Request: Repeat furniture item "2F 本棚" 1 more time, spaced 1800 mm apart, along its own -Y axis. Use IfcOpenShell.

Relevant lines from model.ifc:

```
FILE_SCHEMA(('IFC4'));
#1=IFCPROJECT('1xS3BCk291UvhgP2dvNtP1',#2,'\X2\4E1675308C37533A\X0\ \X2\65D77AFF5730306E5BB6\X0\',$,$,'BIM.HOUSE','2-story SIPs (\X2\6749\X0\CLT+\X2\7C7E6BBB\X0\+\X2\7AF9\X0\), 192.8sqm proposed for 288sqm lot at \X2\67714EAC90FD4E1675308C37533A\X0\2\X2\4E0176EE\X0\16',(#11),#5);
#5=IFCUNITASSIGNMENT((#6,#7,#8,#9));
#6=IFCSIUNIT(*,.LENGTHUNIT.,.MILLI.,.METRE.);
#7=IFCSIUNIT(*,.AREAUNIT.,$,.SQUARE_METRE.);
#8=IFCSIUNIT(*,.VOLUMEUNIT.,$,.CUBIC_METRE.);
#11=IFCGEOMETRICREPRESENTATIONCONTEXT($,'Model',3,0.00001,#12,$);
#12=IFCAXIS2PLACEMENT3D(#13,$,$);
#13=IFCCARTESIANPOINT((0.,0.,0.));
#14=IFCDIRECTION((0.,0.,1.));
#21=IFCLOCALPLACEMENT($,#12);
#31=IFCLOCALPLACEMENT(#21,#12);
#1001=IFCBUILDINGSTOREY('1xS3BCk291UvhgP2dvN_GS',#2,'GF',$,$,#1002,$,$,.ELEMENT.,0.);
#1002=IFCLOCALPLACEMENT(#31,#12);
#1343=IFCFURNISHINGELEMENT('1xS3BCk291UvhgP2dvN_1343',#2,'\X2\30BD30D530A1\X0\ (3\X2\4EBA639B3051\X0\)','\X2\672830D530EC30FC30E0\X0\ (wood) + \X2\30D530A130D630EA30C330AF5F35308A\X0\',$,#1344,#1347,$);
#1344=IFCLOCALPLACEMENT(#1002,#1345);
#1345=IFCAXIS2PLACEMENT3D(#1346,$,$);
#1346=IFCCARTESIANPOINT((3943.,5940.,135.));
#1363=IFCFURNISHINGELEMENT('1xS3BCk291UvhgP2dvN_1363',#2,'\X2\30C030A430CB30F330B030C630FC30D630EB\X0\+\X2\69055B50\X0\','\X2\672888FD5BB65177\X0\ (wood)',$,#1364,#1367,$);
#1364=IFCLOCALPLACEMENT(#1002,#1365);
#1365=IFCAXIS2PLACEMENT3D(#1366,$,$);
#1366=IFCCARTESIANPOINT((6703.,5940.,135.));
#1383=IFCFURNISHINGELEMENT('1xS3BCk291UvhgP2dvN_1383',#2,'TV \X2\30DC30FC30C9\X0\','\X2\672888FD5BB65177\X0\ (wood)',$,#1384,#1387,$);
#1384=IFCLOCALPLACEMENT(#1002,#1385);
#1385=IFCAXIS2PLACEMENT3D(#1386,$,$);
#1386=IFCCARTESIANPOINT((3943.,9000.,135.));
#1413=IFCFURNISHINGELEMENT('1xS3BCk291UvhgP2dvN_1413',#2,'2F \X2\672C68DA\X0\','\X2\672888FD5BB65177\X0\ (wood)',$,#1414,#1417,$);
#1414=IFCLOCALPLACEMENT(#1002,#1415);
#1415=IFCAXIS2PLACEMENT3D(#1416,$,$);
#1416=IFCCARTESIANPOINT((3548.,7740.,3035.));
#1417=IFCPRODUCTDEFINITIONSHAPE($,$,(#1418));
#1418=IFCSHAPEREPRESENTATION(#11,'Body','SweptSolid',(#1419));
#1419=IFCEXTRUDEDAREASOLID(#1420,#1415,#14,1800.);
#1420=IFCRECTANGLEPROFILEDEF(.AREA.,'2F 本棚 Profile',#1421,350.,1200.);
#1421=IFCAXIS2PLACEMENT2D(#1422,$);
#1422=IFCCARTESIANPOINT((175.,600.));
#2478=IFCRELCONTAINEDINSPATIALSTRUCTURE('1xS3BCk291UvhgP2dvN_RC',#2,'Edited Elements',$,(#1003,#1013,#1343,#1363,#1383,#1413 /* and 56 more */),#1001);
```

```python
import ifcopenshell
import ifcopenshell.api.geometry
import ifcopenshell.api.root
import ifcopenshell.util.element
import ifcopenshell.util.placement
import ifcopenshell.util.unit

model = ifcopenshell.open("model.ifc")
unit_scale = ifcopenshell.util.unit.calculate_unit_scale(model)


def reuse_history(source, copy):
    """copy_class also copies each property set's owner history, people and application; keep the originals."""
    for rel in copy.IsDefinedBy:
        if rel.is_a("IfcRelDefinesByProperties") and (history := rel.RelatingPropertyDefinition.OwnerHistory):
            rel.RelatingPropertyDefinition.OwnerHistory = source.OwnerHistory
            ifcopenshell.util.element.remove_deep2(model, history)


source = model.by_guid("1xS3BCk291UvhgP2dvN_1413")
base = ifcopenshell.util.placement.get_local_placement(source.ObjectPlacement)
step = -base[:3, 1] * 1.8 / unit_scale

for i in range(1, 2):
    copy = ifcopenshell.api.root.copy_class(model, product=source)
    copy.Representation = ifcopenshell.util.element.copy_deep(
        model, source.Representation, exclude=["IfcGeometricRepresentationContext", "IfcRepresentationMap"]
    )
    reuse_history(source, copy)
    matrix = base.copy()
    matrix[:3, 3] += i * step
    print("added at", matrix[:3, 3].round(3) + 0.0)
    ifcopenshell.api.geometry.edit_object_placement(model, product=copy, matrix=matrix, is_si=False)

model.write("model_updated.ifc")
```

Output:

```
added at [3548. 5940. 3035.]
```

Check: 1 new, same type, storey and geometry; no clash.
